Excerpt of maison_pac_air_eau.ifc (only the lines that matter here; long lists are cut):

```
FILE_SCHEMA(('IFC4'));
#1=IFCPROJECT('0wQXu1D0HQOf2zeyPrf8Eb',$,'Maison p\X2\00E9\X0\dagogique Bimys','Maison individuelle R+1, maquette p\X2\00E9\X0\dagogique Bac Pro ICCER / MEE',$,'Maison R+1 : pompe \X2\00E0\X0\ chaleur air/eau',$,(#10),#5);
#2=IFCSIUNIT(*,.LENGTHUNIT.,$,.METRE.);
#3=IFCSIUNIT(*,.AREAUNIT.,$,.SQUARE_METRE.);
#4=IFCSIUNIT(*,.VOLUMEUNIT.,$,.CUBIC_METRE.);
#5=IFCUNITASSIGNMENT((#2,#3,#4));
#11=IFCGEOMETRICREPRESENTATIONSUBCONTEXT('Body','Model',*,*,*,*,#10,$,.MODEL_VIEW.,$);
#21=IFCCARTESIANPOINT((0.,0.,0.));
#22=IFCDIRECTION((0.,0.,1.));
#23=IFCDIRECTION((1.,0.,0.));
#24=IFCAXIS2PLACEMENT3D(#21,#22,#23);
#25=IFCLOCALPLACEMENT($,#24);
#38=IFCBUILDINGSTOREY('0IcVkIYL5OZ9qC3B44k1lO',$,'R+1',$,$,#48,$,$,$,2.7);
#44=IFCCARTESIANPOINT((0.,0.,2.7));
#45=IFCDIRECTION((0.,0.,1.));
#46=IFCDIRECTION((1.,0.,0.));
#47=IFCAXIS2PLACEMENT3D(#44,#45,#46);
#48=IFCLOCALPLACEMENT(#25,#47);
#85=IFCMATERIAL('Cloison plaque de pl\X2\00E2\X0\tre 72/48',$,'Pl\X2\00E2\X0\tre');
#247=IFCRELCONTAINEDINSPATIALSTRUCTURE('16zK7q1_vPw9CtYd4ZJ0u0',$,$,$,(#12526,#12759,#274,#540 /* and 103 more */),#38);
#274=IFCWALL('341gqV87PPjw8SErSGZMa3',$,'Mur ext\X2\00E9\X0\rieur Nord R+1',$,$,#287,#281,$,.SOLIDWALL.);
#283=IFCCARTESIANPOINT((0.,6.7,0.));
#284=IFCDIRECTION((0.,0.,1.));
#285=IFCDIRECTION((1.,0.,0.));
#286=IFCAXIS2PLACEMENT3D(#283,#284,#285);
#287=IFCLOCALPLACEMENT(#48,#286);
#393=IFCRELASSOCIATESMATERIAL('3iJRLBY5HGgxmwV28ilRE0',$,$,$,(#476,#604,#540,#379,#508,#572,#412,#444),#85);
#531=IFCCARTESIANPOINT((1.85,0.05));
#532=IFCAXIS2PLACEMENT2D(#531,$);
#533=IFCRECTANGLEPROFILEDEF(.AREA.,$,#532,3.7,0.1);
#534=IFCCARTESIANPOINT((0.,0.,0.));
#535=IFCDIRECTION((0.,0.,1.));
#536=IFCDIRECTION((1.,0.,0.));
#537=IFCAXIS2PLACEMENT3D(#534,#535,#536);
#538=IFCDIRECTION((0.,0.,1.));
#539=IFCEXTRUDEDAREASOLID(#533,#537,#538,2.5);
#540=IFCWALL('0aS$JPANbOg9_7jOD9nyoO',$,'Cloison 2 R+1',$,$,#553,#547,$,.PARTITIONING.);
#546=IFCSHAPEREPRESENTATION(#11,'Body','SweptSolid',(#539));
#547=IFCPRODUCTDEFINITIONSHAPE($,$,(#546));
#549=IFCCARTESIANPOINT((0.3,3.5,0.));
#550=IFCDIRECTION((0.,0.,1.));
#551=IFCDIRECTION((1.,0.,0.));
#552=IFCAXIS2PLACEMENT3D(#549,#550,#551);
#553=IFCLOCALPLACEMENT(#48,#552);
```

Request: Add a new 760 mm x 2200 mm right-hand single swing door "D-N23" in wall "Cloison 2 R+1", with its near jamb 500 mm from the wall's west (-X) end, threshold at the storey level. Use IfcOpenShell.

```python
import numpy as np
import ifcopenshell
import ifcopenshell.api.feature
import ifcopenshell.api.geometry
import ifcopenshell.api.root
import ifcopenshell.api.spatial
import ifcopenshell.geom
import ifcopenshell.util.element
import ifcopenshell.util.placement
import ifcopenshell.util.representation
import ifcopenshell.util.shape
import ifcopenshell.util.unit

model = ifcopenshell.open("maison_pac_air_eau.ifc")
unit_scale = ifcopenshell.util.unit.calculate_unit_scale(model)
settings = ifcopenshell.geom.settings()


def volume(element):
    """Net volume in cubic metres, openings subtracted."""
    shape = ifcopenshell.geom.create_shape(settings, element)
    return ifcopenshell.util.shape.get_volume(shape.geometry)


wall = model.by_guid("0aS$JPANbOg9_7jOD9nyoO")
storey = ifcopenshell.util.element.get_container(wall, ifc_class="IfcBuildingStorey")
context = ifcopenshell.util.representation.get_context(model, "Model", "Body", "MODEL_VIEW")
before = volume(wall)

width, height, from_end, sill = 0.76, 2.2, 0.5, 0.0  # metres

# The wall runs along its own X axis, and the end named is its -X end.
wall_shape = ifcopenshell.geom.create_shape(settings, wall)
x, y, z = ifcopenshell.util.shape.get_vertices(wall_shape.geometry).T
start = x.min() + from_end
face, thickness = float(y.min()), float(y.max() - y.min())
wall_matrix = ifcopenshell.util.placement.get_local_placement(wall.ObjectPlacement)
level = ifcopenshell.util.placement.get_local_placement(storey.ObjectPlacement)[2, 3]


def in_wall(x, y):
    """Placement at x, y metres in the wall's axes, at sill height."""
    matrix = wall_matrix.copy()
    matrix[:, 3] = wall_matrix @ np.array([x / unit_scale, y / unit_scale, 0.0, 1.0])
    matrix[2, 3] = level + sill / unit_scale
    return matrix


# Opening: a box that overshoots both wall faces by 50 mm.
opening = ifcopenshell.api.root.create_entity(model, ifc_class="IfcOpeningElement", predefined_type="OPENING")
box = ifcopenshell.api.geometry.add_wall_representation(
    model, context=context, length=width, height=height, thickness=thickness + 0.1
)
ifcopenshell.api.geometry.assign_representation(model, product=opening, representation=box)
ifcopenshell.api.geometry.edit_object_placement(model, product=opening, matrix=in_wall(start, face - 0.05), is_si=False)
ifcopenshell.api.feature.add_feature(model, feature=opening, element=wall)

door = ifcopenshell.api.root.create_entity(model, ifc_class="IfcDoor", name="D-N23", predefined_type="DOOR")
door.OverallWidth, door.OverallHeight = width / unit_scale, height / unit_scale
door.OperationType = "SINGLE_SWING_RIGHT"
body = ifcopenshell.api.geometry.add_door_representation(
    model,
    context=context,
    overall_width=door.OverallWidth,
    overall_height=door.OverallHeight,
    operation_type="SINGLE_SWING_RIGHT",
    lining_properties={"LiningDepth": thickness / unit_scale, "ThresholdDepth": thickness / unit_scale},
)
ifcopenshell.api.geometry.assign_representation(model, product=door, representation=body)
ifcopenshell.api.spatial.assign_container(model, products=[door], relating_structure=storey)
ifcopenshell.api.feature.add_filling(model, opening=opening, element=door)

# The lining spans the wall, so the door starts at the wall face.
ifcopenshell.api.geometry.edit_object_placement(model, product=door, matrix=in_wall(start, face), is_si=False)

after = volume(wall)

print(f"wall volume {before:.3f} -> {after:.3f} m3")

model.write("maison_pac_air_eau-out.ifc")
```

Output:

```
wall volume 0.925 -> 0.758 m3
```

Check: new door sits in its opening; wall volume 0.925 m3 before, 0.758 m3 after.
